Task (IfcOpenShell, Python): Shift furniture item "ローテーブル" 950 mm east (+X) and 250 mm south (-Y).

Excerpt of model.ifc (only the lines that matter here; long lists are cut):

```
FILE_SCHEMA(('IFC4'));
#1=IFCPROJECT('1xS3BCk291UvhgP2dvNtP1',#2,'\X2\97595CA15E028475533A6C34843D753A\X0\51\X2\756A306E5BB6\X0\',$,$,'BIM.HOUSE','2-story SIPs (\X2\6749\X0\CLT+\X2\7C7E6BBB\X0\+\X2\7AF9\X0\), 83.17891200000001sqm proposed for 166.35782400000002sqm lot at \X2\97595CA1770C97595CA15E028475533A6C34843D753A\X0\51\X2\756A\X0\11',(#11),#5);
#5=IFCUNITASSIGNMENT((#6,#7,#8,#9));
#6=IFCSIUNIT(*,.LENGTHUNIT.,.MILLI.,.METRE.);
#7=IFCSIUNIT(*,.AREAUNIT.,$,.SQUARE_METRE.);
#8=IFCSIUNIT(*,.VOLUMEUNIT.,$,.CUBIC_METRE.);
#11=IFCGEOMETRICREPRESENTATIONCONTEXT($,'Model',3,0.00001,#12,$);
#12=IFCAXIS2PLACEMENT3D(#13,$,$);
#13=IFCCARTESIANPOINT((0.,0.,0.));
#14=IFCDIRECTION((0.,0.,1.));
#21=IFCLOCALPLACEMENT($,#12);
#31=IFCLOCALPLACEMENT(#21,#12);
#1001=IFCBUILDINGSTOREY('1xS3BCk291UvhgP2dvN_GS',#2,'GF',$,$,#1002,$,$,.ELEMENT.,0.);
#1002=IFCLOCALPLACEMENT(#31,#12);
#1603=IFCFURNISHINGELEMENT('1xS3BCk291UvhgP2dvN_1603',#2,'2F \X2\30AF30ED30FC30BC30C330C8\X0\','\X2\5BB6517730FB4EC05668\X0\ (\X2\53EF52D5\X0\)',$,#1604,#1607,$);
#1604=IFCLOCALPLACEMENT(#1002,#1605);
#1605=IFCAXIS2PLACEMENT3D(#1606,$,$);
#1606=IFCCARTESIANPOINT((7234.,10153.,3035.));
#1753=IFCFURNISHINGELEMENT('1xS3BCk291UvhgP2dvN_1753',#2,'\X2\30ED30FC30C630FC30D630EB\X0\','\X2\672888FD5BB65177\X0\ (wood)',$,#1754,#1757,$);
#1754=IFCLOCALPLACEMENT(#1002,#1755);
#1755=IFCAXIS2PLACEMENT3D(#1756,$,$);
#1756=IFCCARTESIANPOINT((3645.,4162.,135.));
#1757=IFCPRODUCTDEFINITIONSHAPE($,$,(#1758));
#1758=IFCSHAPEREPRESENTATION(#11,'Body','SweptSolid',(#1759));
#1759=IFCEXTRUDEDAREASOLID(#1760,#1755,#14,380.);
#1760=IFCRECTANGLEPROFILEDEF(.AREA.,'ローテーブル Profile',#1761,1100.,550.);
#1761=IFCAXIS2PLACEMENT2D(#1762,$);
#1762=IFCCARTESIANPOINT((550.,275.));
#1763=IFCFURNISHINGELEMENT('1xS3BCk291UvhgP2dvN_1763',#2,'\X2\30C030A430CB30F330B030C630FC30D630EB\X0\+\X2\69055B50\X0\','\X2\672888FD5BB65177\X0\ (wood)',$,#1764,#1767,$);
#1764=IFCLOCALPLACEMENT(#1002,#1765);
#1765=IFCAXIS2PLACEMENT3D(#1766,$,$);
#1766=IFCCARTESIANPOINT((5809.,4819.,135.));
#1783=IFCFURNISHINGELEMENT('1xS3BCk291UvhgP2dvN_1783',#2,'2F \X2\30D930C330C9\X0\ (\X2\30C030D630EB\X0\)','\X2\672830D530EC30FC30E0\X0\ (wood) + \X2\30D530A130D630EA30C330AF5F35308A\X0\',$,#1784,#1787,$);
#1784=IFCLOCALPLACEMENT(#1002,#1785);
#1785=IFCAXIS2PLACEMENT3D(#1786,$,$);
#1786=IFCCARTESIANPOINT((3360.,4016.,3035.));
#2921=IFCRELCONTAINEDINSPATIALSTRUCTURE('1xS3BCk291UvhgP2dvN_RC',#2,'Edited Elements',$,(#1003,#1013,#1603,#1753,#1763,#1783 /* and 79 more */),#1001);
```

```python
import ifcopenshell
import ifcopenshell.api.geometry
import ifcopenshell.util.placement
import ifcopenshell.util.unit

model = ifcopenshell.open("model.ifc")
unit_scale = ifcopenshell.util.unit.calculate_unit_scale(model)

item = model.by_id(1753)
matrix = ifcopenshell.util.placement.get_local_placement(item.ObjectPlacement)
matrix[0, 3] += 0.95 / unit_scale
matrix[1, 3] -= 0.25 / unit_scale
ifcopenshell.api.geometry.edit_object_placement(model, product=item, matrix=matrix, is_si=False)

print(ifcopenshell.util.placement.get_local_placement(item.ObjectPlacement).round(3) + 0.0)

model.write("model_v2.ifc")
```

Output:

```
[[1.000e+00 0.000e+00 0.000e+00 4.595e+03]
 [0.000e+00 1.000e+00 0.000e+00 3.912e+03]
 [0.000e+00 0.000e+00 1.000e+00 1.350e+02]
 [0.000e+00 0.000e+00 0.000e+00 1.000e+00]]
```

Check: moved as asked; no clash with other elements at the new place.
